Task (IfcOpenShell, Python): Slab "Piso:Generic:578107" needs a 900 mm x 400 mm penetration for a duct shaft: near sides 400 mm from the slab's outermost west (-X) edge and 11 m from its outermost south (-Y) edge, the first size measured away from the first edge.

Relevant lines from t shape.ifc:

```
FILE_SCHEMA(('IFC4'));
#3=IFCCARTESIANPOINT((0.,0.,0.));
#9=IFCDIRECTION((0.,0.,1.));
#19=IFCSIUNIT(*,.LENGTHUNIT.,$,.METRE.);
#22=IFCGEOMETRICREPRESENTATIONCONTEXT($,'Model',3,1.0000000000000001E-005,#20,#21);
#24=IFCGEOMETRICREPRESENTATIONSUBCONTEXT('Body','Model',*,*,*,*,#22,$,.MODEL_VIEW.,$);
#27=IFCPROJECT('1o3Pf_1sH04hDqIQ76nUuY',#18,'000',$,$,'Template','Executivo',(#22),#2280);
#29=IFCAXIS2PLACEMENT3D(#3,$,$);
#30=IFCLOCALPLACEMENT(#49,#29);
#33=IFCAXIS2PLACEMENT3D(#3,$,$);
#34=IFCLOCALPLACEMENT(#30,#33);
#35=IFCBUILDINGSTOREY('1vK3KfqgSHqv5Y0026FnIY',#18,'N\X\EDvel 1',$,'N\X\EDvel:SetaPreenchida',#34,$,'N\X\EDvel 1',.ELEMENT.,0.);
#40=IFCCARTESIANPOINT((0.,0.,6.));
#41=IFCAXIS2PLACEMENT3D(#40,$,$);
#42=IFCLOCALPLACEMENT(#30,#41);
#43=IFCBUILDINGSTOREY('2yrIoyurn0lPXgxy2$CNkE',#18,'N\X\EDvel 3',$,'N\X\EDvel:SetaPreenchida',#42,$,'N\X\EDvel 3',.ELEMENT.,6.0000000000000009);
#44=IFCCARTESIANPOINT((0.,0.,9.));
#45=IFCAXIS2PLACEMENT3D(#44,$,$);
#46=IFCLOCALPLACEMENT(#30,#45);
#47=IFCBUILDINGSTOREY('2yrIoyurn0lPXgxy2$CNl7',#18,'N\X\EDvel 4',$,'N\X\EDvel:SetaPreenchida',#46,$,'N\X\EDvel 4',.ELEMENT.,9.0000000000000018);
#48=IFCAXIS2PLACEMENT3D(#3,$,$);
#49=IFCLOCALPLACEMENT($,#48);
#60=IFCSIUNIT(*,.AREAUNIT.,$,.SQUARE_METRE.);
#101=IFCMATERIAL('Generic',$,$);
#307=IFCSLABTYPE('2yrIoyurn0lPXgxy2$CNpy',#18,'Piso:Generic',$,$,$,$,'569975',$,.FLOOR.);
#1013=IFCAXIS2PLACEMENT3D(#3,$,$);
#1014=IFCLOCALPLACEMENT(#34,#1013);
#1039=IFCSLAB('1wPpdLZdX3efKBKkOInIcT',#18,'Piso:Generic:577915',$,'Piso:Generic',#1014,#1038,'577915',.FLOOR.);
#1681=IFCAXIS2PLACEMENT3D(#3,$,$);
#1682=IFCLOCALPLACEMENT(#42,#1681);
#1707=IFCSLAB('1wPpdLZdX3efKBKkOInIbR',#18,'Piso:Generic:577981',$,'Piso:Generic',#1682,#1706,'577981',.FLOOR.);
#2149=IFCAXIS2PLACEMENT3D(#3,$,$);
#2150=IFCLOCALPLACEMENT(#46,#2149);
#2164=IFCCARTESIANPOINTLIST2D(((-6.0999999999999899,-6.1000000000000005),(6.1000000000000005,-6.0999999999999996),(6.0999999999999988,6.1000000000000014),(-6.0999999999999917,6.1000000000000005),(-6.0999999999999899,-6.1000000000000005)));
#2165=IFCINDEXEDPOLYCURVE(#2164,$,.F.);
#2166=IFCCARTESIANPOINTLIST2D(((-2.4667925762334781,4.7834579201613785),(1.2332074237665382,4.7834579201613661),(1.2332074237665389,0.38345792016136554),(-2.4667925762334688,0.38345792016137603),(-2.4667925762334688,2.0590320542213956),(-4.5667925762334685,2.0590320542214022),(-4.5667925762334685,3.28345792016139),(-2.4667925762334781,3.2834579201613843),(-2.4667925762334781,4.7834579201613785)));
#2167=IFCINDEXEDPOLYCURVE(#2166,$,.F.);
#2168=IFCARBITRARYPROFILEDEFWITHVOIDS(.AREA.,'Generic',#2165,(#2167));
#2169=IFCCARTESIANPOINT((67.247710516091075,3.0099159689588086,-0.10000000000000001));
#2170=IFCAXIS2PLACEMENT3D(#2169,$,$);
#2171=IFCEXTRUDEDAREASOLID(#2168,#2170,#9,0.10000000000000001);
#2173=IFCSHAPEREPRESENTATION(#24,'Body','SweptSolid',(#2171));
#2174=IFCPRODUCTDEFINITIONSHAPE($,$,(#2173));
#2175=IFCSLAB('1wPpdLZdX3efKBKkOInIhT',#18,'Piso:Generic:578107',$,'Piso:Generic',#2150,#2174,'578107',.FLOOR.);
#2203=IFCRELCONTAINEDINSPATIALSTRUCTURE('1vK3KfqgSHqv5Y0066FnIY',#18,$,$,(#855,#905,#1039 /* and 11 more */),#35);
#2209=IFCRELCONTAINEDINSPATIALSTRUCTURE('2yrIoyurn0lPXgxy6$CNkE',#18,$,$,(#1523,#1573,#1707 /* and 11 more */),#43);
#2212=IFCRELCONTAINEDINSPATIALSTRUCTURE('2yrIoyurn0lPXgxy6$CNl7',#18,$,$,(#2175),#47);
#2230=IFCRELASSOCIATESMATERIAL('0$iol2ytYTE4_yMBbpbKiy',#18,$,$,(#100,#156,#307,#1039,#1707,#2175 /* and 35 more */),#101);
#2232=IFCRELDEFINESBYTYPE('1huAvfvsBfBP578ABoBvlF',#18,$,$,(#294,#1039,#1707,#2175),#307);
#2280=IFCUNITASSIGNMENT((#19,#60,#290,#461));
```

```python
import numpy as np
import ifcopenshell
import ifcopenshell.api.feature
import ifcopenshell.api.geometry
import ifcopenshell.api.root
import ifcopenshell.geom
import ifcopenshell.util.placement
import ifcopenshell.util.representation
import ifcopenshell.util.shape
import ifcopenshell.util.unit

model = ifcopenshell.open("t shape.ifc")
unit_scale = ifcopenshell.util.unit.calculate_unit_scale(model)
settings = ifcopenshell.geom.settings()


def volume(element):
    """Net volume in cubic metres, openings subtracted."""
    shape = ifcopenshell.geom.create_shape(settings, element)
    return ifcopenshell.util.shape.get_volume(shape.geometry)


slab = model.by_guid("1wPpdLZdX3efKBKkOInIhT")
before = volume(slab)

# Extent in the slab's own axes, in metres. The edges named are its -X and -Y sides.
slab_shape = ifcopenshell.geom.create_shape(settings, slab)
vertices = ifcopenshell.util.shape.get_vertices(slab_shape.geometry)
x_min, y_min, bottom = vertices.min(axis=0)
top = vertices[:, 2].max()

opening = ifcopenshell.api.root.create_entity(model, ifc_class="IfcOpeningElement", name="Duct shaft opening", predefined_type="OPENING")
context = ifcopenshell.util.representation.get_context(model, "Model", "Body", "MODEL_VIEW")
width, depth = 0.9, 0.4
outline = [(0.0, 0.0), (width, 0.0), (width, depth), (0.0, depth), (0.0, 0.0)]
# Overshoot both faces by 50 mm so the cut is clean.
shape = ifcopenshell.api.geometry.add_slab_representation(
    model, context=context, depth=top - bottom + 0.1, polyline=outline
)
ifcopenshell.api.geometry.assign_representation(model, product=opening, representation=shape)

matrix = ifcopenshell.util.placement.get_local_placement(slab.ObjectPlacement)
matrix[:, 3] = matrix @ np.append(np.array([x_min + 0.4, y_min + 11, bottom - 0.05]) / unit_scale, 1.0)
ifcopenshell.api.geometry.edit_object_placement(model, product=opening, matrix=matrix, is_si=False)
ifcopenshell.api.feature.add_feature(model, feature=opening, element=slab)

after = volume(slab)

print(f"slab volume {before:.3f} -> {after:.3f} m3")

model.write("t shape-out.ifc")
```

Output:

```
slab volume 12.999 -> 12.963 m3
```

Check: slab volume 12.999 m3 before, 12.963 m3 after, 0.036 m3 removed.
